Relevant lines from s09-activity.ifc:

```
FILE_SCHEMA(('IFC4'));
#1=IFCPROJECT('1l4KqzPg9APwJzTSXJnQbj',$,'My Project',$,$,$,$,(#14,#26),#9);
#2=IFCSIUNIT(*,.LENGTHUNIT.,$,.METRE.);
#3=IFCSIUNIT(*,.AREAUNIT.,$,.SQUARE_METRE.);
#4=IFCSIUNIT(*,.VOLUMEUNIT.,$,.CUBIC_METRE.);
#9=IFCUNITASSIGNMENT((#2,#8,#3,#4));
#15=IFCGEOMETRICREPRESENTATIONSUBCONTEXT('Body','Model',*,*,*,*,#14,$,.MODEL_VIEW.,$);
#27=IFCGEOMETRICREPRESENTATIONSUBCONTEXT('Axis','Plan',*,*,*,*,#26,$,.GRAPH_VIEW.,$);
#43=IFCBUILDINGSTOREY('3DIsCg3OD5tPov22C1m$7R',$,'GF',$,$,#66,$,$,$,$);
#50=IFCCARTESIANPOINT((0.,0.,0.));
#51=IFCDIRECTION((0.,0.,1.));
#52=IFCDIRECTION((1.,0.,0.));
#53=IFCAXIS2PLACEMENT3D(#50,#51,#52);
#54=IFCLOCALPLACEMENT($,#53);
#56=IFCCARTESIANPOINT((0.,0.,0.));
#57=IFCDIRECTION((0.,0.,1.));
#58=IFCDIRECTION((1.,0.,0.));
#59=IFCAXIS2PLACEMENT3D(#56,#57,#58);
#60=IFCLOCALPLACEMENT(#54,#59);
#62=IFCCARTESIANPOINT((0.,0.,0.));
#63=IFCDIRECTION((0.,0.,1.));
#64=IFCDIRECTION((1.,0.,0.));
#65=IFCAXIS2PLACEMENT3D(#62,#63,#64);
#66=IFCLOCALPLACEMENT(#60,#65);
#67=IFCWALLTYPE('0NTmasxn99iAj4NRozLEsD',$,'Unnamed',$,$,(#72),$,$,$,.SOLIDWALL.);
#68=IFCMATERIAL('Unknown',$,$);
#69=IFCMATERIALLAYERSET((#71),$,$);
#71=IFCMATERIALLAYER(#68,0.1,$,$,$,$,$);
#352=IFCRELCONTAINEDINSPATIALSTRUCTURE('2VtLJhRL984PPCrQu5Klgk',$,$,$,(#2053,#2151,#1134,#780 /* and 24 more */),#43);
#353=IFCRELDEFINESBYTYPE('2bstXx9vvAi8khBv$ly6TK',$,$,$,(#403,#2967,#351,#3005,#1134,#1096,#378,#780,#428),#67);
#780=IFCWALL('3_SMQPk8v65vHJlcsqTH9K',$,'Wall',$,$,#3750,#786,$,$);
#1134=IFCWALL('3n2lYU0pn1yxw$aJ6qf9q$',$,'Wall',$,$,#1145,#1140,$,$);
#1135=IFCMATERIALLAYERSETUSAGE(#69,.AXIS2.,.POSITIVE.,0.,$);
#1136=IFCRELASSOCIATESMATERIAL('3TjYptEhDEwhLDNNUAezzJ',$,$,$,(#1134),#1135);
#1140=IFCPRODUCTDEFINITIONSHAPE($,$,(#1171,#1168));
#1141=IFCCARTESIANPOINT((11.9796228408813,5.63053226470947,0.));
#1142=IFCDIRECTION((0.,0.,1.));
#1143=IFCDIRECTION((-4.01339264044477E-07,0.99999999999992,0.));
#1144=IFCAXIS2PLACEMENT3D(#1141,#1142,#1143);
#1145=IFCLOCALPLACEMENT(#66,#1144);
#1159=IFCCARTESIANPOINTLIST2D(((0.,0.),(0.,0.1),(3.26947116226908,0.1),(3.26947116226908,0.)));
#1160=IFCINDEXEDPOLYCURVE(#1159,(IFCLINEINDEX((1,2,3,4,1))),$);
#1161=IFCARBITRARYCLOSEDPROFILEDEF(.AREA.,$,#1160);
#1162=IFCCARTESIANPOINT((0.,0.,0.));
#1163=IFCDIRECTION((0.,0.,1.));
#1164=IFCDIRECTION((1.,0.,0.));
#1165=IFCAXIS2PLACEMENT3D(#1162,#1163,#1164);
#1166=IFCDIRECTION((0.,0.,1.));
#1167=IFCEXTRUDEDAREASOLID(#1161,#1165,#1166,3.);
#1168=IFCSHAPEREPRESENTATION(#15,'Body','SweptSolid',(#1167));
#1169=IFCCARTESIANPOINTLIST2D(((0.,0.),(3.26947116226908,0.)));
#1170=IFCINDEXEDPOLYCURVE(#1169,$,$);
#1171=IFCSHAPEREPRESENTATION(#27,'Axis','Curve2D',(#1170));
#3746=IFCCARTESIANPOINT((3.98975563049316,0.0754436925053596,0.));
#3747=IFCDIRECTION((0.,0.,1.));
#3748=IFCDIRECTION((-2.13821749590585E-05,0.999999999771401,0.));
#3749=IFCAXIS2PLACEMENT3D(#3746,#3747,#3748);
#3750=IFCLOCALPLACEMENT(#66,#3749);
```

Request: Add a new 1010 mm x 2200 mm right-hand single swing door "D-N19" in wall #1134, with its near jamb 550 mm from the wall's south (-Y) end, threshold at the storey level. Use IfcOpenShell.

```python
import numpy as np
import ifcopenshell
import ifcopenshell.api.feature
import ifcopenshell.api.geometry
import ifcopenshell.api.root
import ifcopenshell.api.spatial
import ifcopenshell.geom
import ifcopenshell.util.element
import ifcopenshell.util.placement
import ifcopenshell.util.representation
import ifcopenshell.util.shape
import ifcopenshell.util.unit

model = ifcopenshell.open("s09-activity.ifc")
unit_scale = ifcopenshell.util.unit.calculate_unit_scale(model)
settings = ifcopenshell.geom.settings()


def volume(element):
    """Net volume in cubic metres, openings subtracted."""
    shape = ifcopenshell.geom.create_shape(settings, element)
    return ifcopenshell.util.shape.get_volume(shape.geometry)


wall = model.by_guid("3n2lYU0pn1yxw$aJ6qf9q$")
storey = ifcopenshell.util.element.get_container(wall, ifc_class="IfcBuildingStorey")
context = ifcopenshell.util.representation.get_context(model, "Model", "Body", "MODEL_VIEW")
before = volume(wall)

width, height, from_end, sill = 1.01, 2.2, 0.55, 0.0  # metres

# The wall runs along its own X axis, and the end named is its -X end.
wall_shape = ifcopenshell.geom.create_shape(settings, wall)
x, y, z = ifcopenshell.util.shape.get_vertices(wall_shape.geometry).T
start = x.min() + from_end
face, thickness = float(y.min()), float(y.max() - y.min())
wall_matrix = ifcopenshell.util.placement.get_local_placement(wall.ObjectPlacement)
level = ifcopenshell.util.placement.get_local_placement(storey.ObjectPlacement)[2, 3]


def in_wall(x, y):
    """Placement at x, y metres in the wall's axes, at sill height."""
    matrix = wall_matrix.copy()
    matrix[:, 3] = wall_matrix @ np.array([x / unit_scale, y / unit_scale, 0.0, 1.0])
    matrix[2, 3] = level + sill / unit_scale
    return matrix


# Opening: a box that overshoots both wall faces by 50 mm.
opening = ifcopenshell.api.root.create_entity(model, ifc_class="IfcOpeningElement", predefined_type="OPENING")
box = ifcopenshell.api.geometry.add_wall_representation(
    model, context=context, length=width, height=height, thickness=thickness + 0.1
)
ifcopenshell.api.geometry.assign_representation(model, product=opening, representation=box)
ifcopenshell.api.geometry.edit_object_placement(model, product=opening, matrix=in_wall(start, face - 0.05), is_si=False)
ifcopenshell.api.feature.add_feature(model, feature=opening, element=wall)

door = ifcopenshell.api.root.create_entity(model, ifc_class="IfcDoor", name="D-N19", predefined_type="DOOR")
door.OverallWidth, door.OverallHeight = width / unit_scale, height / unit_scale
door.OperationType = "SINGLE_SWING_RIGHT"
body = ifcopenshell.api.geometry.add_door_representation(
    model,
    context=context,
    overall_width=door.OverallWidth,
    overall_height=door.OverallHeight,
    operation_type="SINGLE_SWING_RIGHT",
    lining_properties={"LiningDepth": thickness / unit_scale, "ThresholdDepth": thickness / unit_scale},
)
ifcopenshell.api.geometry.assign_representation(model, product=door, representation=body)
ifcopenshell.api.spatial.assign_container(model, products=[door], relating_structure=storey)
ifcopenshell.api.feature.add_filling(model, opening=opening, element=door)

# The lining spans the wall, so the door starts at the wall face.
ifcopenshell.api.geometry.edit_object_placement(model, product=door, matrix=in_wall(start, face), is_si=False)

after = volume(wall)

print(f"wall volume {before:.3f} -> {after:.3f} m3")

model.write("s09-activity_updated.ifc")
```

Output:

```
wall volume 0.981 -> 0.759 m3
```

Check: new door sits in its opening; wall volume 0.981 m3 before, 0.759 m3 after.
